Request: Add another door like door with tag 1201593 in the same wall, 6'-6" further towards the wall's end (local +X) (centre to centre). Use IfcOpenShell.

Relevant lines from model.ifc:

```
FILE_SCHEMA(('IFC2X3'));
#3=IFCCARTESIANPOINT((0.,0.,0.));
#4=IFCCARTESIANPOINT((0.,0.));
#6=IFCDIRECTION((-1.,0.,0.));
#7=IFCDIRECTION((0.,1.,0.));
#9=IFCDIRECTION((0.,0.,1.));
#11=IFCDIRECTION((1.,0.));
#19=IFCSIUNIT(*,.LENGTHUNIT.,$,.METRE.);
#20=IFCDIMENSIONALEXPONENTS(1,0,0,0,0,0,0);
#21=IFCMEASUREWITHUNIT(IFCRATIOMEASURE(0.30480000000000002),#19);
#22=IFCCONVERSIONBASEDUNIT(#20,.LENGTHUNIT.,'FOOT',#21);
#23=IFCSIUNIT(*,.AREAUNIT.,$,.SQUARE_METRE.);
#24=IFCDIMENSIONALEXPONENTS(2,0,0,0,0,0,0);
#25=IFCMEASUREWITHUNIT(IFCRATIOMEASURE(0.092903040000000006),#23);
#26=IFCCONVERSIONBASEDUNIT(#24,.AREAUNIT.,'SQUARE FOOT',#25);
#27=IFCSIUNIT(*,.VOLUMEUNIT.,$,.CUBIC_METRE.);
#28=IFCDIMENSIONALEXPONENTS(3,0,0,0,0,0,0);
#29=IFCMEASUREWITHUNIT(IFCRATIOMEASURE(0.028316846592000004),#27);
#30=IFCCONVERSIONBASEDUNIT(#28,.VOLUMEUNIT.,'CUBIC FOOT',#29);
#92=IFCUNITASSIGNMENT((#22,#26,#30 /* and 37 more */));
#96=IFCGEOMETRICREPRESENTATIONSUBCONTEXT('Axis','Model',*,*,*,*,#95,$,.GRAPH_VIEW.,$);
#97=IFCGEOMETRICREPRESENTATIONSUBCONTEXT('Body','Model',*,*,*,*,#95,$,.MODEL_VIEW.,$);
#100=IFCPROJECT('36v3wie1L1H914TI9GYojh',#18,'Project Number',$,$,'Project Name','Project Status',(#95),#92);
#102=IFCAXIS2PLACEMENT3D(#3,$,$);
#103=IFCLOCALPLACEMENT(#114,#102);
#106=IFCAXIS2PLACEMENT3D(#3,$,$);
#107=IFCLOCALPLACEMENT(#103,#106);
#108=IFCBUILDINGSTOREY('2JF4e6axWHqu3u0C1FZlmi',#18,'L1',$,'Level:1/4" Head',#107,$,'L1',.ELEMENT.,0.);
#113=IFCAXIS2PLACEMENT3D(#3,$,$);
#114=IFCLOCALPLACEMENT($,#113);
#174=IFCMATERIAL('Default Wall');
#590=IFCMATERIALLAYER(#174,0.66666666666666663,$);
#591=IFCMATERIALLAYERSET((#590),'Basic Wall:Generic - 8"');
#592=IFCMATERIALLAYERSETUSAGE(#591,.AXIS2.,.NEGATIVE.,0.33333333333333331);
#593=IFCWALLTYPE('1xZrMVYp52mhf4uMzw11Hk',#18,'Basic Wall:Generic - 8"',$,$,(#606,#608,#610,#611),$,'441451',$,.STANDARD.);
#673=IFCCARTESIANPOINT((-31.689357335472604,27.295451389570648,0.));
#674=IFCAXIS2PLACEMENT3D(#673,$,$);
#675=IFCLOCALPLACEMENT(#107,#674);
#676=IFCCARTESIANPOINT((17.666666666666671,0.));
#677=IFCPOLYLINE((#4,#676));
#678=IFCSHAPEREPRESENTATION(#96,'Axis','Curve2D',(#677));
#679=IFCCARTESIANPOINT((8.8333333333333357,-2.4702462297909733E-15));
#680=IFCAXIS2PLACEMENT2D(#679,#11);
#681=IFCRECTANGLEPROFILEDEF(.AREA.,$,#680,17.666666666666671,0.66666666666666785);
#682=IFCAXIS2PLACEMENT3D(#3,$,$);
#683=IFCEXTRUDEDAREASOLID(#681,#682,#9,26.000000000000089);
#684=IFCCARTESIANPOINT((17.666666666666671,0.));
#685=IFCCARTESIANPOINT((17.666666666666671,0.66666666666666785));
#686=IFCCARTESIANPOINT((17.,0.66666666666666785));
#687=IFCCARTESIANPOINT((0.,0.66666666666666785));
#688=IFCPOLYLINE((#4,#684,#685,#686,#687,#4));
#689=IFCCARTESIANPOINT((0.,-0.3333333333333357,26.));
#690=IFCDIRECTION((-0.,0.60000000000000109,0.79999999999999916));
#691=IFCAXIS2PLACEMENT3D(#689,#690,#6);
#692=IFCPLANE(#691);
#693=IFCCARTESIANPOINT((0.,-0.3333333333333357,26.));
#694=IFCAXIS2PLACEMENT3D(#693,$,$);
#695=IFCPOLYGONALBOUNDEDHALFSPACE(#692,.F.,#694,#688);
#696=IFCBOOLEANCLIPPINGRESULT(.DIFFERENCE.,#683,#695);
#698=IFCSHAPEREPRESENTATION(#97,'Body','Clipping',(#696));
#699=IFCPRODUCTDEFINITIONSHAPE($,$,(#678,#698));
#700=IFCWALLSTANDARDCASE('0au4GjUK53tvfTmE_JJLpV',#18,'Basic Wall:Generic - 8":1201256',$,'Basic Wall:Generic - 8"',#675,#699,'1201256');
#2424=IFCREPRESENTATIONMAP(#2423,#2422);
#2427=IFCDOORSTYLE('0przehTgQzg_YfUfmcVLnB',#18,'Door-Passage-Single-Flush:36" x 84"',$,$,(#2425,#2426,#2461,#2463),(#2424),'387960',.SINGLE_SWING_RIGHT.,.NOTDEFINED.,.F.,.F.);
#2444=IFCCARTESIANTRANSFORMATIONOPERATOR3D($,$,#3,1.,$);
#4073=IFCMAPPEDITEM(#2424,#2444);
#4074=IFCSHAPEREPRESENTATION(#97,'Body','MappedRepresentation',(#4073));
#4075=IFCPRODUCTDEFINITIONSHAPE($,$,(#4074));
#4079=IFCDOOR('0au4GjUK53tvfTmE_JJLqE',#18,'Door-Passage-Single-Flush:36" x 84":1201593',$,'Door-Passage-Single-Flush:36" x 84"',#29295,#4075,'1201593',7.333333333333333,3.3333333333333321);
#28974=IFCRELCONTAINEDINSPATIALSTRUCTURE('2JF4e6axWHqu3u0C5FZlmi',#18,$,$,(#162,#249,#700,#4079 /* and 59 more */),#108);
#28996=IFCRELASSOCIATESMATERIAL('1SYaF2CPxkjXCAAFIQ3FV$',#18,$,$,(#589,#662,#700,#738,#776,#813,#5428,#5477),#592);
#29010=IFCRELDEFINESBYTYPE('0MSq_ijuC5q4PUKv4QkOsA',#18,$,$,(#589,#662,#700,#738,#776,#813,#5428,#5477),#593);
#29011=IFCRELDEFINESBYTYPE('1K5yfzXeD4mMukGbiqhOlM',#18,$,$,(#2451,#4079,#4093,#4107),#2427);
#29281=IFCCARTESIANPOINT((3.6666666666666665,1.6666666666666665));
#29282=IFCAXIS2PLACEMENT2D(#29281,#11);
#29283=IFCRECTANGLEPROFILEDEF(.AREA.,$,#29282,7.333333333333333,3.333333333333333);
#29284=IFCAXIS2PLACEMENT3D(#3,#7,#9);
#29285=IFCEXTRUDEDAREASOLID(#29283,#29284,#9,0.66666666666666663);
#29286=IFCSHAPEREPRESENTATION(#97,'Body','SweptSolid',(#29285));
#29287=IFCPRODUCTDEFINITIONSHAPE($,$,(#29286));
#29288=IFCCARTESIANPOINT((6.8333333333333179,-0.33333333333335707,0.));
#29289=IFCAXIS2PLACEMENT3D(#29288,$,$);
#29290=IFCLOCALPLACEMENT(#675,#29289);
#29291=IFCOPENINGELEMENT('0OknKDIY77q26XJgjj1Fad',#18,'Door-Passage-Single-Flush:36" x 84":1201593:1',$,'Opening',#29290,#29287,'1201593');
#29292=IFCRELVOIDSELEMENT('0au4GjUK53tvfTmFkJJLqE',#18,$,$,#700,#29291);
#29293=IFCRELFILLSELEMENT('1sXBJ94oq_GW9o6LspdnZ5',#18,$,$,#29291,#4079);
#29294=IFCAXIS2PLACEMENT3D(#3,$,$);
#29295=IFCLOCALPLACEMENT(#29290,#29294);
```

```python
import ifcopenshell
import ifcopenshell.api.feature
import ifcopenshell.api.geometry
import ifcopenshell.api.root
import ifcopenshell.geom
import ifcopenshell.util.element
import ifcopenshell.util.placement
import ifcopenshell.util.shape
import ifcopenshell.util.unit

model = ifcopenshell.open("model.ifc")
unit_scale = ifcopenshell.util.unit.calculate_unit_scale(model)
settings = ifcopenshell.geom.settings()


def volume(element):
    """Net volume in cubic metres, openings subtracted."""
    shape = ifcopenshell.geom.create_shape(settings, element)
    return ifcopenshell.util.shape.get_volume(shape.geometry)


def reuse_history(source, copy):
    """copy_class also copies each property set's owner history, people and application; keep the originals."""
    for rel in copy.IsDefinedBy:
        if rel.is_a("IfcRelDefinesByProperties") and (history := rel.RelatingPropertyDefinition.OwnerHistory):
            rel.RelatingPropertyDefinition.OwnerHistory = source.OwnerHistory
            ifcopenshell.util.element.remove_deep2(model, history)


door = model.by_id(4079)
opening = door.FillsVoids[0].RelatingOpeningElement
wall = opening.VoidsElements[0].RelatingBuildingElement
before = volume(wall)
shift = ifcopenshell.util.placement.get_local_placement(wall.ObjectPlacement)[:3, 0] * 78 * 0.0254 / unit_scale

# copy_class copies the void relationship, type, container and properties, but no geometry.
new_opening = ifcopenshell.api.root.copy_class(model, product=opening)
new_opening.Representation = ifcopenshell.util.element.copy_deep(
    model, opening.Representation, exclude=["IfcGeometricRepresentationContext", "IfcRepresentationMap"]
)
new_opening.Name = 'Door-Passage-Single-Flush:36" x 84"'
new_opening.Tag = None
new_door = ifcopenshell.api.root.copy_class(model, product=door)
new_door.Representation = ifcopenshell.util.element.copy_deep(
    model, door.Representation, exclude=["IfcGeometricRepresentationContext", "IfcRepresentationMap"]
)
new_door.Name = 'Door-Passage-Single-Flush:36" x 84"'
new_door.Tag = None
reuse_history(door, new_door)
fills = ifcopenshell.api.feature.add_filling(model, opening=new_opening, element=new_door)
fills.OwnerHistory = new_door.OwnerHistory  # required in IFC2X3

for old, new in ((opening, new_opening), (door, new_door)):
    matrix = ifcopenshell.util.placement.get_local_placement(old.ObjectPlacement)
    matrix[:3, 3] += shift
    ifcopenshell.api.geometry.edit_object_placement(model, product=new, matrix=matrix, is_si=False)

after = volume(wall)

print(f"wall volume {before:.3f} -> {after:.3f} m3")

model.write("model_v2.ifc")
```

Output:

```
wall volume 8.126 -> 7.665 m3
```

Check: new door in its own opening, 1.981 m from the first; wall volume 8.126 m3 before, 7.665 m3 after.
